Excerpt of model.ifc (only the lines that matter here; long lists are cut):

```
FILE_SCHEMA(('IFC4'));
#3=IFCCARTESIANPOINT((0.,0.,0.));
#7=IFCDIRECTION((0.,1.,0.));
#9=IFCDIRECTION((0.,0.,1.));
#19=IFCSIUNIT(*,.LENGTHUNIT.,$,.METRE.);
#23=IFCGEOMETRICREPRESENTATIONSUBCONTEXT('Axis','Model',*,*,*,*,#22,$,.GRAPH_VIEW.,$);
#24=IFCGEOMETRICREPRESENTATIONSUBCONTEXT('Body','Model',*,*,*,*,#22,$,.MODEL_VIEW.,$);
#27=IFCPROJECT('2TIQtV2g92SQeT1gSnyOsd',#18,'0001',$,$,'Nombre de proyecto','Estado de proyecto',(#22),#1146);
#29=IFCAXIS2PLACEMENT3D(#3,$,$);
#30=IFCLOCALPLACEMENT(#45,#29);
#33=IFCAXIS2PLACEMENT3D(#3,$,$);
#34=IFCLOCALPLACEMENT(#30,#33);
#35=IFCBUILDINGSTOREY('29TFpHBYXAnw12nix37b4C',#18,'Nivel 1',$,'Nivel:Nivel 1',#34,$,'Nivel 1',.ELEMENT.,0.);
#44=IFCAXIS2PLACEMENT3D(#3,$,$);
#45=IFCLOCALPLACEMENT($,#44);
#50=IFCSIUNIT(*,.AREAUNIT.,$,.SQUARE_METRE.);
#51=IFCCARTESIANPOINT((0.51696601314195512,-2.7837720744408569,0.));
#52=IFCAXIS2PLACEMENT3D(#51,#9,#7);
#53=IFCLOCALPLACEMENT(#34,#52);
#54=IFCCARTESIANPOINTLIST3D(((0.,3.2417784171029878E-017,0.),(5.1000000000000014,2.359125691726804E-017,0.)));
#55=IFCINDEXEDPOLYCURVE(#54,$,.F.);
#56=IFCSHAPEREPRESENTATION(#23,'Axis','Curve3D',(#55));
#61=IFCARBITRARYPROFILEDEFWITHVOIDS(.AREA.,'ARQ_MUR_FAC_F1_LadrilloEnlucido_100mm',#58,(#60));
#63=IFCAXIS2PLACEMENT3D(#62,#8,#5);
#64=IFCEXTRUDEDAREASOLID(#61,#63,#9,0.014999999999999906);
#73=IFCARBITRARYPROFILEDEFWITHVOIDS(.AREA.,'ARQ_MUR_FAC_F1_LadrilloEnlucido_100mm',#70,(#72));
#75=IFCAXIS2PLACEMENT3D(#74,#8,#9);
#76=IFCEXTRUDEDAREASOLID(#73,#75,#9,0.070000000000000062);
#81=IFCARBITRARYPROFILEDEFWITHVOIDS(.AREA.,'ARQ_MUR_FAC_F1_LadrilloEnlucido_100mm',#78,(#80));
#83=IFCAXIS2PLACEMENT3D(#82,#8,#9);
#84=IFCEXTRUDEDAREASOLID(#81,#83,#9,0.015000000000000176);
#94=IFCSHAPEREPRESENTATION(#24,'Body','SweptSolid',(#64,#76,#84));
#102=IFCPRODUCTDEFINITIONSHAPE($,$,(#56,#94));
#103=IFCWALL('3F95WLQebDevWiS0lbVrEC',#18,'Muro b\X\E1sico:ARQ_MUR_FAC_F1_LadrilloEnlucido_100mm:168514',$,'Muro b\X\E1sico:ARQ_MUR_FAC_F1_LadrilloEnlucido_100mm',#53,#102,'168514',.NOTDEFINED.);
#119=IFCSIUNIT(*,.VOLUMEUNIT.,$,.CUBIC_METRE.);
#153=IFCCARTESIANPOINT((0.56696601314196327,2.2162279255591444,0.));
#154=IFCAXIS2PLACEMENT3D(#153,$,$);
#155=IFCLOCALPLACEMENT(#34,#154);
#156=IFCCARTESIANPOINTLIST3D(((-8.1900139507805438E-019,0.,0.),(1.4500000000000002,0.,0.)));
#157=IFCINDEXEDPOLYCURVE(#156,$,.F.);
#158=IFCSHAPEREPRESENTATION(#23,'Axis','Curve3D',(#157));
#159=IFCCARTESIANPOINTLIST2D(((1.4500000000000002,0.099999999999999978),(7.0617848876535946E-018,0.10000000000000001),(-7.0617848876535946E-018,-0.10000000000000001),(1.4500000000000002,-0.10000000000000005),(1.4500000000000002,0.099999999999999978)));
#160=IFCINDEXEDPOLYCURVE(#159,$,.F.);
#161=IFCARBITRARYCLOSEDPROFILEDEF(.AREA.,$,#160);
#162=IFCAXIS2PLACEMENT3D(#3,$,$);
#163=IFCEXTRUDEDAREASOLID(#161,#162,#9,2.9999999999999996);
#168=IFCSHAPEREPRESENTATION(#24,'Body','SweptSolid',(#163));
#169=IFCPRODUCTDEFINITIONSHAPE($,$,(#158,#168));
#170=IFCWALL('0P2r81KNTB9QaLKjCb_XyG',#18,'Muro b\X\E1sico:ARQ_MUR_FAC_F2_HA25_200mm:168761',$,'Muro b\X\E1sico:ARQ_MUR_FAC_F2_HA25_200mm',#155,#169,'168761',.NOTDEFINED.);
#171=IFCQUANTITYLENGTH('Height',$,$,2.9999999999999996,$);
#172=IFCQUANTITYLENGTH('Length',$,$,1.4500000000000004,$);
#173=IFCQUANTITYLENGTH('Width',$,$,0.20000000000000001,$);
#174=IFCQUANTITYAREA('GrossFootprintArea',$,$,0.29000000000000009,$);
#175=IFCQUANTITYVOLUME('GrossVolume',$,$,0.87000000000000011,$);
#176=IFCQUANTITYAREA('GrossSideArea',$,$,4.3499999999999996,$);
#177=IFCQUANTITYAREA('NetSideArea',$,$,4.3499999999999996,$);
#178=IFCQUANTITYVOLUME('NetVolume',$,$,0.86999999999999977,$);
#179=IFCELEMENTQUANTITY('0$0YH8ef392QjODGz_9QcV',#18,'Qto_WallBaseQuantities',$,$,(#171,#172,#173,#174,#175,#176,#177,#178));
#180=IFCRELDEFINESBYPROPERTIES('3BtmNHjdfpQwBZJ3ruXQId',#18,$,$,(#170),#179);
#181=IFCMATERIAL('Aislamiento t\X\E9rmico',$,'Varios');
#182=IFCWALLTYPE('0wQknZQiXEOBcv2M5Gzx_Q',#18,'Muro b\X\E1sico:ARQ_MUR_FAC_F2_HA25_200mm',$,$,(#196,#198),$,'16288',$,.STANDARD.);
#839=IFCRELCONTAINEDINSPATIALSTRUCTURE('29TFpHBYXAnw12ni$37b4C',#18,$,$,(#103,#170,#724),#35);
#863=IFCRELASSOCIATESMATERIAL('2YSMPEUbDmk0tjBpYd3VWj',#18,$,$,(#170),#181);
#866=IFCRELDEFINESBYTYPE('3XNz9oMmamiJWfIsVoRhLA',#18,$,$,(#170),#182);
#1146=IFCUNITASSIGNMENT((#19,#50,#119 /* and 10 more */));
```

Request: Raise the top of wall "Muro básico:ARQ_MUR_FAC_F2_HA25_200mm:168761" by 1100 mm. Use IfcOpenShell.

```python
import ifcopenshell
import ifcopenshell.api.pset
import ifcopenshell.geom
import ifcopenshell.util.element
import ifcopenshell.util.representation
import ifcopenshell.util.shape
import ifcopenshell.util.unit

model = ifcopenshell.open("model.ifc")
unit_scale = ifcopenshell.util.unit.calculate_unit_scale(model)
area_scale = ifcopenshell.util.unit.calculate_unit_scale(model, "AREAUNIT")
volume_scale = ifcopenshell.util.unit.calculate_unit_scale(model, "VOLUMEUNIT")
settings = ifcopenshell.geom.settings()


def volume(element):
    """Net volume in cubic metres, openings subtracted."""
    shape = ifcopenshell.geom.create_shape(settings, element)
    return ifcopenshell.util.shape.get_volume(shape.geometry)


wall = model.by_guid("0P2r81KNTB9QaLKjCb_XyG")
before = volume(wall)

body = ifcopenshell.util.representation.get_representation(wall, "Model", "Body")
solid = body.Items[0]
old_height = solid.Depth
solid.Depth += 1.1 / unit_scale
after = volume(wall)
thickness = 0.2  # wall thickness in metres

# Update the stored height, areas and volumes.
qto = model.by_id(ifcopenshell.util.element.get_pset(wall, "Qto_WallBaseQuantities", should_inherit=False)["id"])
ifcopenshell.api.pset.edit_qto(model, qto=qto, properties={
    "Height": solid.Depth,
    "GrossVolume": ifcopenshell.util.element.get_pset(wall, "Qto_WallBaseQuantities", "GrossVolume") * solid.Depth / old_height,
    "GrossSideArea": ifcopenshell.util.element.get_pset(wall, "Qto_WallBaseQuantities", "GrossSideArea") * solid.Depth / old_height,
    "NetSideArea": after / thickness / area_scale,
    "NetVolume": after / volume_scale,
})

print(f"height {old_height:g} -> {solid.Depth:g}, volume {before:.3f} -> {after:.3f} m3")

model.write("model-out.ifc")
```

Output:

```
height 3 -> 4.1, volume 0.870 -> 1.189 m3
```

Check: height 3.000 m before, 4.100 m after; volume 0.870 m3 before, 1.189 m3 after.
